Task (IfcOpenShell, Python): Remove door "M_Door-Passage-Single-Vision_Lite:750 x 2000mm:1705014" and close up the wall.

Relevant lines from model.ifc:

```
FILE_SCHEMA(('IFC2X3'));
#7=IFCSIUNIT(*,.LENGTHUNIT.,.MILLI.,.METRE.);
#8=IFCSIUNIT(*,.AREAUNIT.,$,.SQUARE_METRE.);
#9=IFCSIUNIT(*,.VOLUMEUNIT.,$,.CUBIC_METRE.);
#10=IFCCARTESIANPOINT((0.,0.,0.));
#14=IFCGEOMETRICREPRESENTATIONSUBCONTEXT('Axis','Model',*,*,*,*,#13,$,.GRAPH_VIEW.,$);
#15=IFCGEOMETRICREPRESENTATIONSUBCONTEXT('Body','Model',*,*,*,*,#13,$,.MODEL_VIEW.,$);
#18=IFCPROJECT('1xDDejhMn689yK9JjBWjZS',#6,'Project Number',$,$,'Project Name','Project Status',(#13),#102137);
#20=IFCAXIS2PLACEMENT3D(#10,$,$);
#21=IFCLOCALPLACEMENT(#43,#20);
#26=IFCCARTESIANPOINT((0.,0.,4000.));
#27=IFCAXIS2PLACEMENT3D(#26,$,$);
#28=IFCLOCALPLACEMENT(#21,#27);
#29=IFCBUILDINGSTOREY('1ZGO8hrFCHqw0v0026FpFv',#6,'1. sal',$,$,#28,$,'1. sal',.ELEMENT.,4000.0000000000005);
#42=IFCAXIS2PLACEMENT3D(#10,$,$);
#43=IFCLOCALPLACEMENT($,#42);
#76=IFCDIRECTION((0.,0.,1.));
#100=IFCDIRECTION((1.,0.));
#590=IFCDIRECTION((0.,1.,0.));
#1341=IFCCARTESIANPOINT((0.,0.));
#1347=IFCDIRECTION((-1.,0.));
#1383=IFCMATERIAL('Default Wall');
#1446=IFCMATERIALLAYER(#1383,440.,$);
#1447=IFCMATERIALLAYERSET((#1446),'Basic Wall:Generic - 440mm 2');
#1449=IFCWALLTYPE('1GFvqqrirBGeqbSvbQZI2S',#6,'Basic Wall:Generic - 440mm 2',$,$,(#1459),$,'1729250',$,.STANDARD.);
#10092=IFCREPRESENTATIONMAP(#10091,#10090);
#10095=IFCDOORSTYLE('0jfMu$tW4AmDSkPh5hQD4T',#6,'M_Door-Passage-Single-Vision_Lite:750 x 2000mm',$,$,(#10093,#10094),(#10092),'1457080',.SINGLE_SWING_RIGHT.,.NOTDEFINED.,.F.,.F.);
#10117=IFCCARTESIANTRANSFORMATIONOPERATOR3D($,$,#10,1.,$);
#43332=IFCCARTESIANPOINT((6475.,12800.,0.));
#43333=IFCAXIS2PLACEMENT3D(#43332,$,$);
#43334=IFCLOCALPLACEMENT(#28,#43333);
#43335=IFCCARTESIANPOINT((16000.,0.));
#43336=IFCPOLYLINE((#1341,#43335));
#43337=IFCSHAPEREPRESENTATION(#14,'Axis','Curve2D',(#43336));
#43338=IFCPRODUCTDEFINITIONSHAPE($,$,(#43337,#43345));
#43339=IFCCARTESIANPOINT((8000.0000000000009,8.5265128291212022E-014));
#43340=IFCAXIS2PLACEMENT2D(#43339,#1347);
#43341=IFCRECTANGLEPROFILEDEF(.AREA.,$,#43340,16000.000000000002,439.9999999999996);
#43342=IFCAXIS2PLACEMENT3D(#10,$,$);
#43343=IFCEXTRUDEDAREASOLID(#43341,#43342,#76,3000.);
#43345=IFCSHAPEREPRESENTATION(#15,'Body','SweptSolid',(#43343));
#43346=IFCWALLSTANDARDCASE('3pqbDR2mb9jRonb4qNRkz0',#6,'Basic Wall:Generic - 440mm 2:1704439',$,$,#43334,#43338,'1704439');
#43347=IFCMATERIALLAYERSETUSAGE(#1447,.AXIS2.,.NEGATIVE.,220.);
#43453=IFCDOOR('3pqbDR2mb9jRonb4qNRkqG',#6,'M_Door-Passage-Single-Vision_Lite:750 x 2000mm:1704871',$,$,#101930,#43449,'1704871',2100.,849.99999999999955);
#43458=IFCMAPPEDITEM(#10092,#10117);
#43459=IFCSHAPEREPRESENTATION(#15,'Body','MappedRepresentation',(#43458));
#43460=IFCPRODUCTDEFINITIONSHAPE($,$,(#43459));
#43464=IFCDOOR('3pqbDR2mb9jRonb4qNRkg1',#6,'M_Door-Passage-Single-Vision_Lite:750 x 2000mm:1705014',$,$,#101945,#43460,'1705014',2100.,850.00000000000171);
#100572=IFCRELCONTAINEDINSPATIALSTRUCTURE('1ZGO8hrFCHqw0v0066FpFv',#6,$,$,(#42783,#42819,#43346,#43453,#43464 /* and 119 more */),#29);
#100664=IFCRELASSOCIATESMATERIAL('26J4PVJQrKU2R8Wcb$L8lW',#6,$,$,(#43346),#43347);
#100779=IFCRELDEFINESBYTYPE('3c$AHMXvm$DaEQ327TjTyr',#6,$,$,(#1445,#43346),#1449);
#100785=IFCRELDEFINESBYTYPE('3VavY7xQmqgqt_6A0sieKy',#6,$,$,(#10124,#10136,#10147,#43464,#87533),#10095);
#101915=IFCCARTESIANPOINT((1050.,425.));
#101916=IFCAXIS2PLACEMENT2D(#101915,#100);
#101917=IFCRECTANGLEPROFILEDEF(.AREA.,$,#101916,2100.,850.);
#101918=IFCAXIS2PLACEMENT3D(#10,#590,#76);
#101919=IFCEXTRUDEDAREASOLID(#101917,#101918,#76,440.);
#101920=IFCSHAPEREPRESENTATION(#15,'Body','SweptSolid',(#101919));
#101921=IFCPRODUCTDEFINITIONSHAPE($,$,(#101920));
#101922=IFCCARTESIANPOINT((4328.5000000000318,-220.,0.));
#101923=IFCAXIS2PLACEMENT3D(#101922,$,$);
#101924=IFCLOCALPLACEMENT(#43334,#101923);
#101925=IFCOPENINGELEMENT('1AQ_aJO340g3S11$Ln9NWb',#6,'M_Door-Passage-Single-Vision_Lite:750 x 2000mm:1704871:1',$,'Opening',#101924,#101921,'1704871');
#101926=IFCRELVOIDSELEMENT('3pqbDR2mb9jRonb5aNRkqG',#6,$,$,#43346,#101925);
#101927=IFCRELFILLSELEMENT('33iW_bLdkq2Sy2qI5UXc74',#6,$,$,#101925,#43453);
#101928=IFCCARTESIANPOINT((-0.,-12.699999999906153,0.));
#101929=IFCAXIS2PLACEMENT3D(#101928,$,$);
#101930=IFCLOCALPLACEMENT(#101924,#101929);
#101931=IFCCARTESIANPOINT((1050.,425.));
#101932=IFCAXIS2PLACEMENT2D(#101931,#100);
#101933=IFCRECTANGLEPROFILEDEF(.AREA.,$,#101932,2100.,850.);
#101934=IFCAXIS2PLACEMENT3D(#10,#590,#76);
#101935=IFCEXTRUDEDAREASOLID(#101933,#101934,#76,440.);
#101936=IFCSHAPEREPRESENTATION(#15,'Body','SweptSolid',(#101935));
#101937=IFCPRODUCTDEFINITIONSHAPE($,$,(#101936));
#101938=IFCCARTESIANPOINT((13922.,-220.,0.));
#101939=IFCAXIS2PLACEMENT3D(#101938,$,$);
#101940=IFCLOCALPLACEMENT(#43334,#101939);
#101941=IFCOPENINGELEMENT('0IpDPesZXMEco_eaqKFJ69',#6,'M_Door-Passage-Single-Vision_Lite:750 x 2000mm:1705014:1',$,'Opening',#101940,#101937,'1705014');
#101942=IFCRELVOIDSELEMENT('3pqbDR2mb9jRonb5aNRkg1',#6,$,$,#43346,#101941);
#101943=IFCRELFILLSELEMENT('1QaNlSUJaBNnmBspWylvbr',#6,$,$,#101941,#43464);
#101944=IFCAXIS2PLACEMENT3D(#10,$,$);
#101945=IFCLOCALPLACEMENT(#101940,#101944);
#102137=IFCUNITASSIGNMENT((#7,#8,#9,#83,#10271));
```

```python
import ifcopenshell
import ifcopenshell.api.feature
import ifcopenshell.api.root
import ifcopenshell.geom
import ifcopenshell.util.shape

model = ifcopenshell.open("model.ifc")
settings = ifcopenshell.geom.settings()


def volume(element):
    """Net volume in cubic metres, openings subtracted."""
    shape = ifcopenshell.geom.create_shape(settings, element)
    return ifcopenshell.util.shape.get_volume(shape.geometry)


door = model.by_id(43464)
opening = door.FillsVoids[0].RelatingOpeningElement
wall = opening.VoidsElements[0].RelatingBuildingElement
before = volume(wall)

ifcopenshell.api.root.remove_product(model, product=door)
ifcopenshell.api.feature.remove_feature(model, feature=opening)

after = volume(wall)

print(f"wall volume {before:.3f} -> {after:.3f} m3")

model.write("model_updated.ifc")
```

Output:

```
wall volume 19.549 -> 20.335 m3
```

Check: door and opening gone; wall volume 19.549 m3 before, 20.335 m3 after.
